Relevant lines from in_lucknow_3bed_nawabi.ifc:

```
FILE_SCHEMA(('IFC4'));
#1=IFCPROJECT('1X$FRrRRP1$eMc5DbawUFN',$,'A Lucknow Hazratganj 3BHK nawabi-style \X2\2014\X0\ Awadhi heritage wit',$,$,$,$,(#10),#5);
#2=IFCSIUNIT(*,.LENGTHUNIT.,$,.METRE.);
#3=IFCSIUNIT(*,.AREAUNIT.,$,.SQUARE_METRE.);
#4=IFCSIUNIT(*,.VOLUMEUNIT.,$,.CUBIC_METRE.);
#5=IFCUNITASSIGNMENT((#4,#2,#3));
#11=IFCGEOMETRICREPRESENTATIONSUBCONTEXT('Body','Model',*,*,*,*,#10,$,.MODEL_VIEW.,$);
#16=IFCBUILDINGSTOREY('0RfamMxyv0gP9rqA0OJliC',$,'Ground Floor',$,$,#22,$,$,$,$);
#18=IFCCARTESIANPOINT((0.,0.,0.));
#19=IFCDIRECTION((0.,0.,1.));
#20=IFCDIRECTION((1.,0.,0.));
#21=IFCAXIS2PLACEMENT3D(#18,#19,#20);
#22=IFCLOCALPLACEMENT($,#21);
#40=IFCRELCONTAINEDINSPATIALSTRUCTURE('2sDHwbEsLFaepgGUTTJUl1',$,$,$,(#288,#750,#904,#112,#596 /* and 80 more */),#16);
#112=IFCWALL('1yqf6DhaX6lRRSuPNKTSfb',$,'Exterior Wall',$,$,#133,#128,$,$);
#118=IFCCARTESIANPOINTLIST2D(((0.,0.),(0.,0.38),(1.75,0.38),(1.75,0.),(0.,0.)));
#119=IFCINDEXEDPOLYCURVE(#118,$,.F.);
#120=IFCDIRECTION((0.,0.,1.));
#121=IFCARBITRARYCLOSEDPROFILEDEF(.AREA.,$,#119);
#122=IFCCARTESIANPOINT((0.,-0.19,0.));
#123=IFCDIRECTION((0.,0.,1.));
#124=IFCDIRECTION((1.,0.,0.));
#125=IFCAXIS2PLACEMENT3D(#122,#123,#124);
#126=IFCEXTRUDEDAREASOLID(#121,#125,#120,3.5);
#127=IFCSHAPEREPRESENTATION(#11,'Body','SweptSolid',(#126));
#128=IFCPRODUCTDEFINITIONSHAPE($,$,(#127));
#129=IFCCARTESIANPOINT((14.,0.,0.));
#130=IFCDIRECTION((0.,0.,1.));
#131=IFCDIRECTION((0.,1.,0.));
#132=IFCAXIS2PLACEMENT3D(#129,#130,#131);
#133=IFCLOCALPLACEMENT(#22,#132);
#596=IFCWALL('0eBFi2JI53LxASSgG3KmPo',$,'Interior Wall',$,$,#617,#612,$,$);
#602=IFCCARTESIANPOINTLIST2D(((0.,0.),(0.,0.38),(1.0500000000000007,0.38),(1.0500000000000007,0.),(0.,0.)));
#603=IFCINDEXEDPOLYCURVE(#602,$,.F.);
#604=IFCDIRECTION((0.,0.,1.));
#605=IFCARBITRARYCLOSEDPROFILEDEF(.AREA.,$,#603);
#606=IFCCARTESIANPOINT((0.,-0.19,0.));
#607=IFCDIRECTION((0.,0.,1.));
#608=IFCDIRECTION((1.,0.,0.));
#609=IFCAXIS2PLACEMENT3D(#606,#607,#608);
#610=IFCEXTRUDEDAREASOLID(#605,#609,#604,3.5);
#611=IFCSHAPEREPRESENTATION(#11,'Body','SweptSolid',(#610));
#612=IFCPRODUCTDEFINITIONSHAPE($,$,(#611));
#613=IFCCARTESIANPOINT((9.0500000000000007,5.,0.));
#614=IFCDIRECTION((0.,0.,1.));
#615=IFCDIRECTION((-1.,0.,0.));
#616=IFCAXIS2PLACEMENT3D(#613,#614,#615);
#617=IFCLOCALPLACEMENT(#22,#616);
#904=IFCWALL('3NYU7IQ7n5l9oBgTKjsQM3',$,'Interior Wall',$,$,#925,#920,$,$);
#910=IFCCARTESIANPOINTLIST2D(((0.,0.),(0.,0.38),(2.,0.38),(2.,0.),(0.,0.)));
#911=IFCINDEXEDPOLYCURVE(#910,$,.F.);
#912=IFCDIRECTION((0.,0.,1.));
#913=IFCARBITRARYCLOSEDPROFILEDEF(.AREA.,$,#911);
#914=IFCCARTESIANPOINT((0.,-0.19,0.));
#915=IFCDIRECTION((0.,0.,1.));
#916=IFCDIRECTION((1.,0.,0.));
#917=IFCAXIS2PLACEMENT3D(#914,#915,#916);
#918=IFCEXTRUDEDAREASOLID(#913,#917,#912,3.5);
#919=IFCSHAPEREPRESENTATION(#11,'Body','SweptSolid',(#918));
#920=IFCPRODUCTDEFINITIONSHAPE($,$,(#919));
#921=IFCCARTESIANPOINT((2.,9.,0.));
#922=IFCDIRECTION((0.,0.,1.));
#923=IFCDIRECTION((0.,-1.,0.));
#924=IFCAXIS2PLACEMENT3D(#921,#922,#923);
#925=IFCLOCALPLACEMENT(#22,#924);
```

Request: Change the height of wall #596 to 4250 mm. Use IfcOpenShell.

```python
import ifcopenshell
import ifcopenshell.geom
import ifcopenshell.util.representation
import ifcopenshell.util.shape

model = ifcopenshell.open("in_lucknow_3bed_nawabi.ifc")
settings = ifcopenshell.geom.settings()


def volume(element):
    """Net volume in cubic metres, openings subtracted."""
    shape = ifcopenshell.geom.create_shape(settings, element)
    return ifcopenshell.util.shape.get_volume(shape.geometry)


wall = model.by_guid("0eBFi2JI53LxASSgG3KmPo")
before = volume(wall)

body = ifcopenshell.util.representation.get_representation(wall, "Model", "Body")
solid = body.Items[0]
old_height = solid.Depth
solid.Depth = 4.25
after = volume(wall)

print(f"height {old_height:g} -> {solid.Depth:g}, volume {before:.3f} -> {after:.3f} m3")

model.write("in_lucknow_3bed_nawabi_edited.ifc")
```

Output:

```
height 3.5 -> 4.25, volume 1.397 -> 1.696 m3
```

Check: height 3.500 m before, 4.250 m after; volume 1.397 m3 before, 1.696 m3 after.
